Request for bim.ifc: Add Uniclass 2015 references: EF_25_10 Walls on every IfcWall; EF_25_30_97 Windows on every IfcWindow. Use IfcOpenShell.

First a look at what the model holds.

```python
import ifcopenshell

model = ifcopenshell.open("bim.ifc")
print(model.schema)
print("classifications:", [c.Name for c in model.by_type("IfcClassification")])
for ifc_class in ("IfcDoor", "IfcRoof", "IfcStair", "IfcWall", "IfcWindow"):
    print(ifc_class, len(model.by_type(ifc_class)))
```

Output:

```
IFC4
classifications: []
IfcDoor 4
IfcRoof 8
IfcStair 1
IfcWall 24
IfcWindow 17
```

```python
import ifcopenshell
import ifcopenshell.api.classification

model = ifcopenshell.open("bim.ifc")

system = ifcopenshell.api.classification.add_classification(model, classification="Uniclass 2015")

codes = {
    "IfcWall": ("EF_25_10", "Walls"),
    "IfcWindow": ("EF_25_30_97", "Windows"),
}
for ifc_class, (code, name) in codes.items():
    products = model.by_type(ifc_class)
    ifcopenshell.api.classification.add_reference(
        model, products=products, classification=system, identification=code, name=name
    )
    print(code, len(products))

model.write("bim_rev.ifc")
```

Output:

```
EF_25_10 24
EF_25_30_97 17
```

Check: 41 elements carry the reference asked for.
